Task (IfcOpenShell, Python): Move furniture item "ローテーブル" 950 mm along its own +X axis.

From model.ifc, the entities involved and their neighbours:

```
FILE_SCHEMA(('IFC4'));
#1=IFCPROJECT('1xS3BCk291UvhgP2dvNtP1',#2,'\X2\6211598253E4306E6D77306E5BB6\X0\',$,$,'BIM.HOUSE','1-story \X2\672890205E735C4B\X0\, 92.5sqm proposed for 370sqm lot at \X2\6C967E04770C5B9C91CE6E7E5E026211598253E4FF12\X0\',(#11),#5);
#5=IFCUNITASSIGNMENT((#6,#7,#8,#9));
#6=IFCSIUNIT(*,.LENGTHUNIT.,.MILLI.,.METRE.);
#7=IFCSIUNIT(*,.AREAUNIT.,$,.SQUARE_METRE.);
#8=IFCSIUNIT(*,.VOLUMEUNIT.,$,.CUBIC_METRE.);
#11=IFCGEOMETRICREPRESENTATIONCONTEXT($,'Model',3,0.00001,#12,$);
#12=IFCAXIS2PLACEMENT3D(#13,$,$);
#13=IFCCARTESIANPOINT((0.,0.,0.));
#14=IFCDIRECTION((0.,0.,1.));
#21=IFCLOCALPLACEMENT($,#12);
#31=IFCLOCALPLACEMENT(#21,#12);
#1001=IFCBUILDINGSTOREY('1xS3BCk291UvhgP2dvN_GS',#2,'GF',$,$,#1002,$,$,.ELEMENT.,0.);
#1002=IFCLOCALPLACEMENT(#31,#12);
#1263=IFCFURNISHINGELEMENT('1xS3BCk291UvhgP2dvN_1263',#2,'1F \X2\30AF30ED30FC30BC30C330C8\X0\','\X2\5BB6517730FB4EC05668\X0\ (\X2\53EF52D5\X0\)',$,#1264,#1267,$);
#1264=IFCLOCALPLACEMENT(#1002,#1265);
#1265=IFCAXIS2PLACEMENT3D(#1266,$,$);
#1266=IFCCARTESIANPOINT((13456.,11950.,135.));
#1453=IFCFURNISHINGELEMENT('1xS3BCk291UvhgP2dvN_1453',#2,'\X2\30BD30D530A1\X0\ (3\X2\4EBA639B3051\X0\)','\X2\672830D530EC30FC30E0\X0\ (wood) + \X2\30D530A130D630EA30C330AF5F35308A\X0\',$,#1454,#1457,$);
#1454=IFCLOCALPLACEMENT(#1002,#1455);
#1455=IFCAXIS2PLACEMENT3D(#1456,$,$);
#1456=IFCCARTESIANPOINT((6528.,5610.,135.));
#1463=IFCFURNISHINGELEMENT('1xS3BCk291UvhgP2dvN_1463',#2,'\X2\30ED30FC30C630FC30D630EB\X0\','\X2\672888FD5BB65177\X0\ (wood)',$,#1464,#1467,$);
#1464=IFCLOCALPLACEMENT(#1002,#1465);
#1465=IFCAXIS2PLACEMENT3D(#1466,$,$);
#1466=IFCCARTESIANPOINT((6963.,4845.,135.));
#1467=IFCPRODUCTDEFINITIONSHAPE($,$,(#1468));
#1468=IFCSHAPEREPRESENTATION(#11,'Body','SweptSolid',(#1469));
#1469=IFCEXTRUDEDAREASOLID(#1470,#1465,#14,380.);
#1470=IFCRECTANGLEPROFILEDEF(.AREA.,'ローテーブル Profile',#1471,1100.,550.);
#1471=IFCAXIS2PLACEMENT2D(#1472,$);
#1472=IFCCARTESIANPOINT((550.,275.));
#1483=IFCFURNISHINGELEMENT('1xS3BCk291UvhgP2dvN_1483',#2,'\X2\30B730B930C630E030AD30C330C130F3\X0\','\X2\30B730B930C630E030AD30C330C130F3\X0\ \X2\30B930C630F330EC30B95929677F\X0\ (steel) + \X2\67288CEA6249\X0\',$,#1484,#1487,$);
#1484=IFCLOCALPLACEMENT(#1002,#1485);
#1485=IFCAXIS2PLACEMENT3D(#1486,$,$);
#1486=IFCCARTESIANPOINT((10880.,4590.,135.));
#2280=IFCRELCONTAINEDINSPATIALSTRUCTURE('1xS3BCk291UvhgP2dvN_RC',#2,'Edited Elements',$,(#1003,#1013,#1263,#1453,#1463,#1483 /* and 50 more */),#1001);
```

```python
import ifcopenshell
import ifcopenshell.api.geometry
import ifcopenshell.util.placement
import ifcopenshell.util.unit

model = ifcopenshell.open("model.ifc")
unit_scale = ifcopenshell.util.unit.calculate_unit_scale(model)

item = model.by_guid("1xS3BCk291UvhgP2dvN_1463")
matrix = ifcopenshell.util.placement.get_local_placement(item.ObjectPlacement)
matrix[:3, 3] += matrix[:3, 0] * 0.95 / unit_scale
ifcopenshell.api.geometry.edit_object_placement(model, product=item, matrix=matrix, is_si=False)

print(ifcopenshell.util.placement.get_local_placement(item.ObjectPlacement).round(3) + 0.0)

model.write("model_v2.ifc")
```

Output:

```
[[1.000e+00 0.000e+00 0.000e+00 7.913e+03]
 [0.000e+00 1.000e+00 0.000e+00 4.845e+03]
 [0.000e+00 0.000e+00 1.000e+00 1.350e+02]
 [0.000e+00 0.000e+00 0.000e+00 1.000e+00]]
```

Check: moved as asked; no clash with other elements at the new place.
